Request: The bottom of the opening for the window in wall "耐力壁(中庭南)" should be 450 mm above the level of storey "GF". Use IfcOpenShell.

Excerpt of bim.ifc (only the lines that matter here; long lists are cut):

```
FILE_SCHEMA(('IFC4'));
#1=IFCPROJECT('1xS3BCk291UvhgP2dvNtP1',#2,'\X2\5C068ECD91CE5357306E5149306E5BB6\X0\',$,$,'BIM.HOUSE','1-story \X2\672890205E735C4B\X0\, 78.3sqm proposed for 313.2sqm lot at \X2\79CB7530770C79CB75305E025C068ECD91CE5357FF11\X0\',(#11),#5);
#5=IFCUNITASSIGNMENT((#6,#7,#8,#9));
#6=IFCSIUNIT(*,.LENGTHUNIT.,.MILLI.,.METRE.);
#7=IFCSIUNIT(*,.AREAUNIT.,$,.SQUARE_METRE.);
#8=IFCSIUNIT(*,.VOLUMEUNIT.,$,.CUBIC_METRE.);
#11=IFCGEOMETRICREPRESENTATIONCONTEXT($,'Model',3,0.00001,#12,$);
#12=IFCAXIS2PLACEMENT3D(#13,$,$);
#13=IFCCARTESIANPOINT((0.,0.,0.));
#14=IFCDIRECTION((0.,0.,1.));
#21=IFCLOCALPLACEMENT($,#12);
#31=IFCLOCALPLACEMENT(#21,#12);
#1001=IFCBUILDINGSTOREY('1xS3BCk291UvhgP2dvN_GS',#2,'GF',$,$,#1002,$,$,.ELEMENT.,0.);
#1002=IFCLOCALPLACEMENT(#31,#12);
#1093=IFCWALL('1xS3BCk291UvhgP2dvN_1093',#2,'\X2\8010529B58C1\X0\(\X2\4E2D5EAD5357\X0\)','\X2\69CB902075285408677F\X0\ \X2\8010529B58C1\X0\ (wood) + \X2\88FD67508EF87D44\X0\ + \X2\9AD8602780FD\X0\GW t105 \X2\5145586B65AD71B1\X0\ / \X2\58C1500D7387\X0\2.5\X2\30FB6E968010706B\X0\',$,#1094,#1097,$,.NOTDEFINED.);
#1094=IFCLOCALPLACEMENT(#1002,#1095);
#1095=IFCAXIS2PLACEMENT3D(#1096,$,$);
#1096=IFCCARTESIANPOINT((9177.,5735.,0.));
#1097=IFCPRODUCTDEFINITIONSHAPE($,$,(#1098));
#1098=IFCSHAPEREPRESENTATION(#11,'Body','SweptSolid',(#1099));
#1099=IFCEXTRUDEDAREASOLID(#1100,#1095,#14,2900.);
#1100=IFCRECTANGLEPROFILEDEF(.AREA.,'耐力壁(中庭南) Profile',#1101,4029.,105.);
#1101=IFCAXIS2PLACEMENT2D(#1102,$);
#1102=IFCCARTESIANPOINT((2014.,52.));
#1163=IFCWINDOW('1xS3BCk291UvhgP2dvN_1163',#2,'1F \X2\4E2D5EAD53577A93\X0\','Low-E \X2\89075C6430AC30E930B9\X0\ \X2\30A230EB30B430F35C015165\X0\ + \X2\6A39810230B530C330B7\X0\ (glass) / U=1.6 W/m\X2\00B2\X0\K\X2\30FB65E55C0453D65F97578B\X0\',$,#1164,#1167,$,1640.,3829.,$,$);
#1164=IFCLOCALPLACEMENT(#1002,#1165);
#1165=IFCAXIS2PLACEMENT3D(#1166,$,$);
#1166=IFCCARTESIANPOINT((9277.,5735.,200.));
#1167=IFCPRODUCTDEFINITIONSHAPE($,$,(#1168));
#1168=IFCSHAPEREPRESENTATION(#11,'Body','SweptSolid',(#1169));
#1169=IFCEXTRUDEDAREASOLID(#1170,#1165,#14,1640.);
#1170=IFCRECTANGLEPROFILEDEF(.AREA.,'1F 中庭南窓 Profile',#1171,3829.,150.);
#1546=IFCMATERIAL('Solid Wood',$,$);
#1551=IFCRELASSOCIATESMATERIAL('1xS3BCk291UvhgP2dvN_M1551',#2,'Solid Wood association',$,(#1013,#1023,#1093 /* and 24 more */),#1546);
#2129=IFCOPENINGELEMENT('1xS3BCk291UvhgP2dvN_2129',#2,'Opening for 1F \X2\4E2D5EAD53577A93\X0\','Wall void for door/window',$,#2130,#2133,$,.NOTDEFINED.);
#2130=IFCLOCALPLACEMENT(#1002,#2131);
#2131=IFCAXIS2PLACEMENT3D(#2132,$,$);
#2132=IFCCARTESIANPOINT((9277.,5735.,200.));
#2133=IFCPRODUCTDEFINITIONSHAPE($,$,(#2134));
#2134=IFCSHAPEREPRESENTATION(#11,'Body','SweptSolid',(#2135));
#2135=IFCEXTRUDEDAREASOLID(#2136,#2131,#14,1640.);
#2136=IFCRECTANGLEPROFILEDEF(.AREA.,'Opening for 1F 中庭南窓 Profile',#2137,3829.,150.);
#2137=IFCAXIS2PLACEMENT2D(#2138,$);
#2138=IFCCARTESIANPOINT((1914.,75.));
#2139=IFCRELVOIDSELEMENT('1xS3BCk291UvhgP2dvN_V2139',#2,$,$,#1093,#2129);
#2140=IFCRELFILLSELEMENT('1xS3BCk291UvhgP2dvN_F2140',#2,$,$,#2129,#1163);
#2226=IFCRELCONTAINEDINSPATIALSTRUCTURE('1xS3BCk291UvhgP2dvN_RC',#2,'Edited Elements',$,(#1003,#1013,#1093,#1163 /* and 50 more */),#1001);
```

```python
import numpy as np
import ifcopenshell
import ifcopenshell.api.geometry
import ifcopenshell.geom
import ifcopenshell.util.element
import ifcopenshell.util.placement
import ifcopenshell.util.shape
import ifcopenshell.util.unit

model = ifcopenshell.open("bim.ifc")
unit_scale = ifcopenshell.util.unit.calculate_unit_scale(model)

window = model.by_guid("1xS3BCk291UvhgP2dvN_1163")
opening = window.FillsVoids[0].RelatingOpeningElement
storey = ifcopenshell.util.element.get_container(window, ifc_class="IfcBuildingStorey")
level = ifcopenshell.util.placement.get_local_placement(storey.ObjectPlacement)[2, 3]

# The opening's origin need not be at the sill, so measure its lowest point.
shape = ifcopenshell.geom.create_shape(ifcopenshell.geom.settings(), opening)
bottom = ifcopenshell.util.shape.get_shape_bottom_elevation(shape, shape.geometry) / unit_scale
dz = level + 0.45 / unit_scale - bottom

shift = np.array([0.0, 0.0, dz])
# The window is not placed relative to its opening, so move both.
for product in (opening, window):
    matrix = ifcopenshell.util.placement.get_local_placement(product.ObjectPlacement)
    matrix[:3, 3] += shift
    ifcopenshell.api.geometry.edit_object_placement(model, product=product, matrix=matrix, is_si=False)

print(f"moved by {dz * unit_scale:+.3f} m")

model.write("bim-out.ifc")
```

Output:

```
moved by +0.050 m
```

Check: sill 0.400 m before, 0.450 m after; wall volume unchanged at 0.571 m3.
